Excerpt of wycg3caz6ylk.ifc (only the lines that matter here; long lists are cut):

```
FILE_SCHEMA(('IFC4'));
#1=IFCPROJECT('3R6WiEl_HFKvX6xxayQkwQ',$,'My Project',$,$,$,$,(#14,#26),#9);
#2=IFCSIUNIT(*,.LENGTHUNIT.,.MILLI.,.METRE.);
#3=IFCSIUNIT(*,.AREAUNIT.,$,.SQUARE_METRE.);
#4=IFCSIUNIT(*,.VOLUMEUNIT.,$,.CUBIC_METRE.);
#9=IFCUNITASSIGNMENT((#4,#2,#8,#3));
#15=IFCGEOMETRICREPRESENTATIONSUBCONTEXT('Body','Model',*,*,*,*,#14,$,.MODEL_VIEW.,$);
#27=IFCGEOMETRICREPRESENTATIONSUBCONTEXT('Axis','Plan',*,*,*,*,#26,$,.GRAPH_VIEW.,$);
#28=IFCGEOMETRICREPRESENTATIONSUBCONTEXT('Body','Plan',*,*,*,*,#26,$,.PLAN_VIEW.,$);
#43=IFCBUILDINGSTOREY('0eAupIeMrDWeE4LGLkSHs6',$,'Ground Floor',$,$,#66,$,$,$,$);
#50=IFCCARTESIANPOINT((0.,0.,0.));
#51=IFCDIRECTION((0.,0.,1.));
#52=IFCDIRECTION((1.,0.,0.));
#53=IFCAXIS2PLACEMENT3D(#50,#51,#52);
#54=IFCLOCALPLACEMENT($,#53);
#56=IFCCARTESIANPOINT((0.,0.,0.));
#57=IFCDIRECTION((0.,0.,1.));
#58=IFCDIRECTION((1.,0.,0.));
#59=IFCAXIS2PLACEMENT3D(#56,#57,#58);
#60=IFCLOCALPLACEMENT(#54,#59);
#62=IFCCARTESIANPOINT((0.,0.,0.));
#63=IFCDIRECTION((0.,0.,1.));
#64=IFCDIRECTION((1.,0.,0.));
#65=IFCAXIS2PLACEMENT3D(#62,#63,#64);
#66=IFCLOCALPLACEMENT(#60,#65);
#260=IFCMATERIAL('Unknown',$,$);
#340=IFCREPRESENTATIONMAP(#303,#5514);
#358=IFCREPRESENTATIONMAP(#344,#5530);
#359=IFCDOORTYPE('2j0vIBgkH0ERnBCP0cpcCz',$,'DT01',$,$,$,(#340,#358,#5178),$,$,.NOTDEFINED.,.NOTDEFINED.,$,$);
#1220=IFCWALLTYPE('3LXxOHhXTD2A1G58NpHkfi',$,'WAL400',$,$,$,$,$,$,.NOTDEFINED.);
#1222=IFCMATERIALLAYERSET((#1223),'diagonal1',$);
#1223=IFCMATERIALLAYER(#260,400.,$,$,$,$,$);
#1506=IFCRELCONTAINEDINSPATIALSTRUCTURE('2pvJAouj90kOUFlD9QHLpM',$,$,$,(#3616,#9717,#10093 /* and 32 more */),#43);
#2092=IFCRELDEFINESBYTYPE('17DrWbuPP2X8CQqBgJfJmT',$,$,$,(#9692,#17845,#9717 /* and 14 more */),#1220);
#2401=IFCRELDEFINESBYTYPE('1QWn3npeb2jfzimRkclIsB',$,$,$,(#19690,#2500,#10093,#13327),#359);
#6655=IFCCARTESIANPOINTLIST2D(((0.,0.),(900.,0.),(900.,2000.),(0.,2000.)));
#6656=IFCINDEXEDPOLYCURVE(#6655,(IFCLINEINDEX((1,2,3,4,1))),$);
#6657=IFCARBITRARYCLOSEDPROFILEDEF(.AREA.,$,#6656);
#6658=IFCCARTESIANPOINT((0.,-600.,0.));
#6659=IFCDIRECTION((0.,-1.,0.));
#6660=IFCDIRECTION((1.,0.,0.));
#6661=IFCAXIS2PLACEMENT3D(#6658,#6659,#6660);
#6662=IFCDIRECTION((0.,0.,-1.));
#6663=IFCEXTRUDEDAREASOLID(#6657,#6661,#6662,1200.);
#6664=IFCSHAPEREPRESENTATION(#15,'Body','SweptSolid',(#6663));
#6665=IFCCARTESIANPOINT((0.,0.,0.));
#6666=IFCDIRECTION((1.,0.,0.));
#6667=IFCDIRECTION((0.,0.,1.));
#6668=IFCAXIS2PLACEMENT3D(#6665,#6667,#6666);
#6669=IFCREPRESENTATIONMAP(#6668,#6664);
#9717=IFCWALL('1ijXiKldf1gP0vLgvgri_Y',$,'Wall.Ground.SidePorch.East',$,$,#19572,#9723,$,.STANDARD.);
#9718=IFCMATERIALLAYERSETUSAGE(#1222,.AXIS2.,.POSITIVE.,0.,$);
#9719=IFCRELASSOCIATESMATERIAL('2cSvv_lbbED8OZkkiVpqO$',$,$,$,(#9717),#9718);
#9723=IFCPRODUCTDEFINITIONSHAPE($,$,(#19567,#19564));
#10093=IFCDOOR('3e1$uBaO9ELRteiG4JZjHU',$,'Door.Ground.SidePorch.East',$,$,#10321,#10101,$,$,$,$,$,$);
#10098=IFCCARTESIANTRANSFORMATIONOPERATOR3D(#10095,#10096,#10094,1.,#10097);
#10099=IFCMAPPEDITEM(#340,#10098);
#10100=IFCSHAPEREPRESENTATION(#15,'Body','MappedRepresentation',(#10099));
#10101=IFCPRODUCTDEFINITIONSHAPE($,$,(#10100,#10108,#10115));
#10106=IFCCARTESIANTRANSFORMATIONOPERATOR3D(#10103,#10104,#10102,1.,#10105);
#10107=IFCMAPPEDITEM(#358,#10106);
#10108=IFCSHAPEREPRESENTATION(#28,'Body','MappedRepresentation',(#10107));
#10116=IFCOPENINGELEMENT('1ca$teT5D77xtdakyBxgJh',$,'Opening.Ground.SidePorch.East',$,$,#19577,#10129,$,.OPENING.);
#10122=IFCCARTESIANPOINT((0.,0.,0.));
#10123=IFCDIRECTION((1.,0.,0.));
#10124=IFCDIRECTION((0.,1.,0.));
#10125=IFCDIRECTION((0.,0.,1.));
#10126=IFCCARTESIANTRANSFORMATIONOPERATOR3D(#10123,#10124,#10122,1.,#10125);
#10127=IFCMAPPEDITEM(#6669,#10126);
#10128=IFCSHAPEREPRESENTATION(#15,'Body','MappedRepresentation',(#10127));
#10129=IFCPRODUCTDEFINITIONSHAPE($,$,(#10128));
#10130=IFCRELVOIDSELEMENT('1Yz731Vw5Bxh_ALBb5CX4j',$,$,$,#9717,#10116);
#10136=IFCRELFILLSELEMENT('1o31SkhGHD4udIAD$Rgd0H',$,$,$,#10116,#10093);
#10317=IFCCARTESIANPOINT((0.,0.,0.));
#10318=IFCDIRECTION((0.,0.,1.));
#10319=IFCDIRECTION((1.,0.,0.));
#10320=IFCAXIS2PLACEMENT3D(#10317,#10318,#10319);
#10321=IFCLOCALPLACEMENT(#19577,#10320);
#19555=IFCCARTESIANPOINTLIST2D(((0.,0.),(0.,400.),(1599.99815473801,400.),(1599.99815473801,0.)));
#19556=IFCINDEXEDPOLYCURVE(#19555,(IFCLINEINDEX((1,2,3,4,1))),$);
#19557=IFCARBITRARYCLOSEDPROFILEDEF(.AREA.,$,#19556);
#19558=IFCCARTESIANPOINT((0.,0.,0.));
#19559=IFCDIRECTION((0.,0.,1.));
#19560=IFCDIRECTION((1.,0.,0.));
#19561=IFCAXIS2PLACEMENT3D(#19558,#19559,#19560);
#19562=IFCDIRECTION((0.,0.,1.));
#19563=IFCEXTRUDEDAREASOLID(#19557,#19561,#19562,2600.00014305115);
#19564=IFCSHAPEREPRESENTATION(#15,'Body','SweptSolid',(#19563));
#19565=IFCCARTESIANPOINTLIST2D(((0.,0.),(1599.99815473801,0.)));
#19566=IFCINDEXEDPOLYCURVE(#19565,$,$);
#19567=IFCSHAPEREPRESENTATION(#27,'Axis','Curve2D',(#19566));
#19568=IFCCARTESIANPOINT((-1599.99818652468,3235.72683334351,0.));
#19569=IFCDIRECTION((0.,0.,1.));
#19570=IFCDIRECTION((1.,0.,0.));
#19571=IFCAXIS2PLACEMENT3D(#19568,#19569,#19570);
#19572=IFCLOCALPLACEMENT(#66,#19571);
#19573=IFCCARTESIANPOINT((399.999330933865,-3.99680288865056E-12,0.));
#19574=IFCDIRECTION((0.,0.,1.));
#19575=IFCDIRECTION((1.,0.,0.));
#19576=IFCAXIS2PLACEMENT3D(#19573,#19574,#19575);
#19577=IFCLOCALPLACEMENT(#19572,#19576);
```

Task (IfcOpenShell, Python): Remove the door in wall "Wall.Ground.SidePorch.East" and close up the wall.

```python
import ifcopenshell
import ifcopenshell.api.feature
import ifcopenshell.api.root
import ifcopenshell.geom
import ifcopenshell.util.shape

model = ifcopenshell.open("wycg3caz6ylk.ifc")
settings = ifcopenshell.geom.settings()


def volume(element):
    """Net volume in cubic metres, openings subtracted."""
    shape = ifcopenshell.geom.create_shape(settings, element)
    return ifcopenshell.util.shape.get_volume(shape.geometry)


door = model.by_guid("3e1$uBaO9ELRteiG4JZjHU")
opening = door.FillsVoids[0].RelatingOpeningElement
wall = opening.VoidsElements[0].RelatingBuildingElement
before = volume(wall)

ifcopenshell.api.root.remove_product(model, product=door)
ifcopenshell.api.feature.remove_feature(model, feature=opening)

after = volume(wall)

print(f"wall volume {before:.3f} -> {after:.3f} m3")

model.write("wycg3caz6ylk_rev.ifc")
```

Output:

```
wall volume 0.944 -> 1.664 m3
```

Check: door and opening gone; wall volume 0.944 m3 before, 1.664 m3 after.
